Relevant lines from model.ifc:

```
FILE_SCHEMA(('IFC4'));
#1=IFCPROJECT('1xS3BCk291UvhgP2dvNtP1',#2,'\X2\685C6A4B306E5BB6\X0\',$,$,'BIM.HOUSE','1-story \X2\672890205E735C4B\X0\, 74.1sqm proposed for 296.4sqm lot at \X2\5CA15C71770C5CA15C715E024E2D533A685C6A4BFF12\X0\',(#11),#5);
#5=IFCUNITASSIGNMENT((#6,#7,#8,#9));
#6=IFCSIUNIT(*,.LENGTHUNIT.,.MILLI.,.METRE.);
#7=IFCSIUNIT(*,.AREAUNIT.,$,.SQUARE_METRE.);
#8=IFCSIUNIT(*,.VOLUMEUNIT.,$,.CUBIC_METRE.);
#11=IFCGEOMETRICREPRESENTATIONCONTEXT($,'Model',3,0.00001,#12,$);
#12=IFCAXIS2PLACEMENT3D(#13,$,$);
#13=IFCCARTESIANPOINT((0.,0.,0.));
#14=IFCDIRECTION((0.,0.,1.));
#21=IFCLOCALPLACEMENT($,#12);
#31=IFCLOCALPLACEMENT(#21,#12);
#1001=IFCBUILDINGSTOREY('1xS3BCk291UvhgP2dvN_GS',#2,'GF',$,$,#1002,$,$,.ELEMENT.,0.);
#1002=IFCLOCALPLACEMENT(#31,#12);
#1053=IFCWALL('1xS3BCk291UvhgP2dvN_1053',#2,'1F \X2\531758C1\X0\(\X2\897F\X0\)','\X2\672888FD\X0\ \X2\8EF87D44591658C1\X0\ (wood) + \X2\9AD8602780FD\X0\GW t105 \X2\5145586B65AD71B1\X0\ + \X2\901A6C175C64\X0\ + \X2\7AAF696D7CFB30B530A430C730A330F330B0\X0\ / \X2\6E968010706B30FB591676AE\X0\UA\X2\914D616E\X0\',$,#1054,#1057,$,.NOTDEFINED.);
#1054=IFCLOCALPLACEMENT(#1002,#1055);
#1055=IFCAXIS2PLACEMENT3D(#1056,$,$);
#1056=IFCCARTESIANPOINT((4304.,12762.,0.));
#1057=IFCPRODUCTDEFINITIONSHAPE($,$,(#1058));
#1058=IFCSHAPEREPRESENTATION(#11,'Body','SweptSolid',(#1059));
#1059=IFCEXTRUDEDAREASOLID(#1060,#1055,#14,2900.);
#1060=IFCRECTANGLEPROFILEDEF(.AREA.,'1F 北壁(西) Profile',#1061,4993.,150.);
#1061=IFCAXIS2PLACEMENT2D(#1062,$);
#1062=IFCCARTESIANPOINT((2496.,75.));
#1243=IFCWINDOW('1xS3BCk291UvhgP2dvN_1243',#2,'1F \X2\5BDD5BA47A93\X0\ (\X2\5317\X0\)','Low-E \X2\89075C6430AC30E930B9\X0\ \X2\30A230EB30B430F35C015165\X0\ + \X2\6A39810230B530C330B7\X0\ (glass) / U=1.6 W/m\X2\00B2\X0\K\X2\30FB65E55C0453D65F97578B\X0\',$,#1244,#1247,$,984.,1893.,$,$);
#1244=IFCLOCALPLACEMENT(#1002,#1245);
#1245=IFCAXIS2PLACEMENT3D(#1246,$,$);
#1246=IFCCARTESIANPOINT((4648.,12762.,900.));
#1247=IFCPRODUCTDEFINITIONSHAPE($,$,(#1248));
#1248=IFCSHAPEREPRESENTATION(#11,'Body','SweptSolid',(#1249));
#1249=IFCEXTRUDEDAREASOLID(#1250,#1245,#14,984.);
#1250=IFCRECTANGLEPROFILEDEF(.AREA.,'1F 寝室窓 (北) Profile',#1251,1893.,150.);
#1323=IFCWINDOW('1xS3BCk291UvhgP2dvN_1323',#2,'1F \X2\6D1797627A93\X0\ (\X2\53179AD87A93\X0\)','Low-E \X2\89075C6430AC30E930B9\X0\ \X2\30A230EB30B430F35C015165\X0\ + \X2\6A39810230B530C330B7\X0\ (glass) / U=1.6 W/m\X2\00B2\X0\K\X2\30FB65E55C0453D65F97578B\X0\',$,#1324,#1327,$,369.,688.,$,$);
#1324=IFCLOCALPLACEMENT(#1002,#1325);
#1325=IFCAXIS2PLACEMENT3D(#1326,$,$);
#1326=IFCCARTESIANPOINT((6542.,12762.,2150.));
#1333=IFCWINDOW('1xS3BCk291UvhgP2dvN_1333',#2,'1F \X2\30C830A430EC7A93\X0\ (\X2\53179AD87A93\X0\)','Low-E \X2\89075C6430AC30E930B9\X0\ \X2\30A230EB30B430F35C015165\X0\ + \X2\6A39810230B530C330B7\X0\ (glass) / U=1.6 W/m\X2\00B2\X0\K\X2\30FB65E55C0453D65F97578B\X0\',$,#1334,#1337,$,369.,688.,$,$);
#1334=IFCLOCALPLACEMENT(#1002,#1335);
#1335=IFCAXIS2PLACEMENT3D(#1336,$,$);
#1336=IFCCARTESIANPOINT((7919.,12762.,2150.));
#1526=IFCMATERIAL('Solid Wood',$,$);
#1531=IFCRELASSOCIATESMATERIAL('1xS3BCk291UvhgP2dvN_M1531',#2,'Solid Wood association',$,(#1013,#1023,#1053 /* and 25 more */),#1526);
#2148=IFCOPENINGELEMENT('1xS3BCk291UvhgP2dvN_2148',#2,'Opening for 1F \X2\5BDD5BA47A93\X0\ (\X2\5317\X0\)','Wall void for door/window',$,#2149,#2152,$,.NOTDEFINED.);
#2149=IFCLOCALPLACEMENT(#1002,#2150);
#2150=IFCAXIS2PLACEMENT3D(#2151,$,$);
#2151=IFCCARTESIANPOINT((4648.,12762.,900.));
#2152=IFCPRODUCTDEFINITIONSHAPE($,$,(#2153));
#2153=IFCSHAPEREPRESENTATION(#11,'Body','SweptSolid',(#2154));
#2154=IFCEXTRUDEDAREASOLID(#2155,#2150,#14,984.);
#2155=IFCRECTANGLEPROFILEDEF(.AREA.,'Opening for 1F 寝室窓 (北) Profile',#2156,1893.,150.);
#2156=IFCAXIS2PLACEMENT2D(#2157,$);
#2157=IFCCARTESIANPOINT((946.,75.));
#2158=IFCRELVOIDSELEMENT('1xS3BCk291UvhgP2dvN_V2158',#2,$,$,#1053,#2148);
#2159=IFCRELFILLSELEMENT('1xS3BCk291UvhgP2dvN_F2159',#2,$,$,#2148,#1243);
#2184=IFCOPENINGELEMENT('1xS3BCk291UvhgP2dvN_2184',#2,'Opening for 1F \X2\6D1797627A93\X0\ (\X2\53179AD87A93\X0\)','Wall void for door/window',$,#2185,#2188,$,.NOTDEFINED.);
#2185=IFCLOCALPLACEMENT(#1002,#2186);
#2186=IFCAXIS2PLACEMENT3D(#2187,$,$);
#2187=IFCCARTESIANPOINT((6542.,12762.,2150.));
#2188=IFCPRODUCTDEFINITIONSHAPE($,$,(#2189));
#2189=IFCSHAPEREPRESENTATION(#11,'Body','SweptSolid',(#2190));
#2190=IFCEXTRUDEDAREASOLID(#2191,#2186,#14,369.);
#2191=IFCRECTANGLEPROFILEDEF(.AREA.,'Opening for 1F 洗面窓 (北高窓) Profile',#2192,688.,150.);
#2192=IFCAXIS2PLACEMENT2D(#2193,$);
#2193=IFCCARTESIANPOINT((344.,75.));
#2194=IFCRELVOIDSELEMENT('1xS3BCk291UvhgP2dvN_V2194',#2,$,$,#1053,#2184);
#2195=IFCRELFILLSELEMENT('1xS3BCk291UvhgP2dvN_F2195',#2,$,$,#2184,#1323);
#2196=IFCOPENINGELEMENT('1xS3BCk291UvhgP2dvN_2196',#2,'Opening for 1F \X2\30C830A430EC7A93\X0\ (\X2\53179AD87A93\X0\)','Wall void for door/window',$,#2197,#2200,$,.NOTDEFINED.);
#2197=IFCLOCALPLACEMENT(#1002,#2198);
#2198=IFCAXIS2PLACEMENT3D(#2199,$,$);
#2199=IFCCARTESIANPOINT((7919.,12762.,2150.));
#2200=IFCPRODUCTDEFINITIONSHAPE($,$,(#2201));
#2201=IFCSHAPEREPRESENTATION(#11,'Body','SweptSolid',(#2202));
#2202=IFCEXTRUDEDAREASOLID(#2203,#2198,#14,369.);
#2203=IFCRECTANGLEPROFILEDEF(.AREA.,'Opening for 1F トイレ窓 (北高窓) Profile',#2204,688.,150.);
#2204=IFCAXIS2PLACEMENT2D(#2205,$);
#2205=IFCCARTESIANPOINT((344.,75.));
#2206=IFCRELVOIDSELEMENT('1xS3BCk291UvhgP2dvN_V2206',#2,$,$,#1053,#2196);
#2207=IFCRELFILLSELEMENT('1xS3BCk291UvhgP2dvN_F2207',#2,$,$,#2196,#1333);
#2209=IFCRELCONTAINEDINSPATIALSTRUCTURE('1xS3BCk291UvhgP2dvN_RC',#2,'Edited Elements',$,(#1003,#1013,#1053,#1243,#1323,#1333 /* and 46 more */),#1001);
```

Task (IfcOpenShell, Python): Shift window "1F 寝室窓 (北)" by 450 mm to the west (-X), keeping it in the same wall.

```python
import ifcopenshell
import ifcopenshell.api.geometry
import ifcopenshell.util.placement

model = ifcopenshell.open("model.ifc")

window = model.by_id(1243)
opening = window.FillsVoids[0].RelatingOpeningElement
wall = opening.VoidsElements[0].RelatingBuildingElement

wall_matrix = ifcopenshell.util.placement.get_local_placement(wall.ObjectPlacement)
shift = wall_matrix[:3, 0] * -450.0
before = ifcopenshell.util.placement.get_local_placement(window.ObjectPlacement)[:3, 3].copy()

# The window is not placed relative to its opening, so move both.
for product in (opening, window):
    matrix = ifcopenshell.util.placement.get_local_placement(product.ObjectPlacement)
    matrix[:3, 3] += shift
    ifcopenshell.api.geometry.edit_object_placement(model, product=product, matrix=matrix, is_si=False)

after = ifcopenshell.util.placement.get_local_placement(window.ObjectPlacement)[:3, 3]
print("window moved by", (after - before).round(3) + 0.0)

model.write("model-out.ifc")
```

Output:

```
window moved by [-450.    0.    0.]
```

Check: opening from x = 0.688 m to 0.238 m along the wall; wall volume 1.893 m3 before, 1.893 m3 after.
